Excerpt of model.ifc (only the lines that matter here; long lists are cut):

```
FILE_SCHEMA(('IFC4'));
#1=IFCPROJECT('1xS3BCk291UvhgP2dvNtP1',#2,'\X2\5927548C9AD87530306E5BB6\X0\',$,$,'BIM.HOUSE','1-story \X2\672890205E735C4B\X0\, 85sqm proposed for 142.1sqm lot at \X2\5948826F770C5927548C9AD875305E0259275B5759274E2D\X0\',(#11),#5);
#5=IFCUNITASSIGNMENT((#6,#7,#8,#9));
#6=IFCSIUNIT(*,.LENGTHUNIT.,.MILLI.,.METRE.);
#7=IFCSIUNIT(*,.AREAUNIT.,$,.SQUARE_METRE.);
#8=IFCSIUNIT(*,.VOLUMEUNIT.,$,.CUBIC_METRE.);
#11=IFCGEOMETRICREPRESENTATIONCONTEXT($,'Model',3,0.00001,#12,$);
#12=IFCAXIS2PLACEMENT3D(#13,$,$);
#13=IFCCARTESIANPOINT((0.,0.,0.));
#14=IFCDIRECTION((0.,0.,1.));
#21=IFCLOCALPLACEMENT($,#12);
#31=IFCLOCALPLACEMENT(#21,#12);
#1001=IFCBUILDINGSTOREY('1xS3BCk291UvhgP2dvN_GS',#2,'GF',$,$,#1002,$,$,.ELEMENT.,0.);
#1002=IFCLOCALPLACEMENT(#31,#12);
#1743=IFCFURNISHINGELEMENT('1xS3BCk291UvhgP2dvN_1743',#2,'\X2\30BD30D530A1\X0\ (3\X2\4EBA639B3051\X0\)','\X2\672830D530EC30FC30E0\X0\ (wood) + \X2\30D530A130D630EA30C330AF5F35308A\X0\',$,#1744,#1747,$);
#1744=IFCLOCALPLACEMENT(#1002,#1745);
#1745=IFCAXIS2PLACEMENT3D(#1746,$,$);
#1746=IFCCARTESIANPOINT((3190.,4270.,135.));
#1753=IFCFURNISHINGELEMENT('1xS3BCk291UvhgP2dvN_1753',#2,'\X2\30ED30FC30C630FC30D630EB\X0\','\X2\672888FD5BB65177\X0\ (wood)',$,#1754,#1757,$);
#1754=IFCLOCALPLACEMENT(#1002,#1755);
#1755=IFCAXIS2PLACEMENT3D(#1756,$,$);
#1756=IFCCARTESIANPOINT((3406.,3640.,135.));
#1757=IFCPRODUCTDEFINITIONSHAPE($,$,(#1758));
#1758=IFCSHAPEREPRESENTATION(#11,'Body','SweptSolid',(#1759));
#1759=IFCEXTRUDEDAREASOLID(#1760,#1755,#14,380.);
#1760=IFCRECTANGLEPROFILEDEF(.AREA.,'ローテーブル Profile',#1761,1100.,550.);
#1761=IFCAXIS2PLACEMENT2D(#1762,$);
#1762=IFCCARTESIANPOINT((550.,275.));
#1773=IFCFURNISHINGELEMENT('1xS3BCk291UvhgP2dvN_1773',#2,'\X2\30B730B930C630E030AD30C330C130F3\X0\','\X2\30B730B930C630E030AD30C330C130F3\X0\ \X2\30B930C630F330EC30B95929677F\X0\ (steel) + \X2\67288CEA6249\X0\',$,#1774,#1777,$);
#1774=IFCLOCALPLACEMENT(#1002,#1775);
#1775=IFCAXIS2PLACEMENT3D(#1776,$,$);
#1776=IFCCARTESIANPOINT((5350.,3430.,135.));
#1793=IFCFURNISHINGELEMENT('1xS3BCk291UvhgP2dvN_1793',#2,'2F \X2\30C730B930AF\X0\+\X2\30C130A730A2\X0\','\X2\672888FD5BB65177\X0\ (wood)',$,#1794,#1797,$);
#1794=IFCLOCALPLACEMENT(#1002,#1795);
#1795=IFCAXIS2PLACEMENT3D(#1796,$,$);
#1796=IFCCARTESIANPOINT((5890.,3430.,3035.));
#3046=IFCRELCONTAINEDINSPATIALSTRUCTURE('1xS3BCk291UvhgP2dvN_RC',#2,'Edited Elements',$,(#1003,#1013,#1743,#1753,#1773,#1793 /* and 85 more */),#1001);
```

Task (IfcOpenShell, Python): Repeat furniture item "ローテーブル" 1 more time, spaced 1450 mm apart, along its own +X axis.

```python
import ifcopenshell
import ifcopenshell.api.geometry
import ifcopenshell.api.root
import ifcopenshell.util.element
import ifcopenshell.util.placement
import ifcopenshell.util.unit

model = ifcopenshell.open("model.ifc")
unit_scale = ifcopenshell.util.unit.calculate_unit_scale(model)


def reuse_history(source, copy):
    """copy_class also copies each property set's owner history, people and application; keep the originals."""
    for rel in copy.IsDefinedBy:
        if rel.is_a("IfcRelDefinesByProperties") and (history := rel.RelatingPropertyDefinition.OwnerHistory):
            rel.RelatingPropertyDefinition.OwnerHistory = source.OwnerHistory
            ifcopenshell.util.element.remove_deep2(model, history)


source = model.by_guid("1xS3BCk291UvhgP2dvN_1753")
base = ifcopenshell.util.placement.get_local_placement(source.ObjectPlacement)
step = base[:3, 0] * 1.45 / unit_scale

for i in range(1, 2):
    copy = ifcopenshell.api.root.copy_class(model, product=source)
    copy.Representation = ifcopenshell.util.element.copy_deep(
        model, source.Representation, exclude=["IfcGeometricRepresentationContext", "IfcRepresentationMap"]
    )
    reuse_history(source, copy)
    matrix = base.copy()
    matrix[:3, 3] += i * step
    print("added at", matrix[:3, 3].round(3) + 0.0)
    ifcopenshell.api.geometry.edit_object_placement(model, product=copy, matrix=matrix, is_si=False)

model.write("model_rev.ifc")
```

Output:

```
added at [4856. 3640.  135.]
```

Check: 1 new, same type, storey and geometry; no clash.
